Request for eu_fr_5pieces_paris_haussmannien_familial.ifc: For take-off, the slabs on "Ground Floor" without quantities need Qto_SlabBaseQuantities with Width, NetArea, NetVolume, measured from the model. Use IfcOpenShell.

First a look at what the model holds.

```python
import ifcopenshell
import ifcopenshell.util.element
import ifcopenshell.util.unit

model = ifcopenshell.open("eu_fr_5pieces_paris_haussmannien_familial.ifc")
print(model.schema)
for unit_type in ("LENGTHUNIT", "AREAUNIT", "VOLUMEUNIT"):
    print(unit_type, ifcopenshell.util.unit.calculate_unit_scale(model, unit_type))
storey = next(s for s in model.by_type("IfcBuildingStorey") if s.Name == "Ground Floor")
slabs = [e for e in ifcopenshell.util.element.get_decomposition(storey) if e.is_a("IfcSlab")]
for e in sorted(slabs, key=lambda e: e.id()):
    print(e.id(), e.is_a(), e.Name, list(ifcopenshell.util.element.get_psets(e, qtos_only=True)), sep=" | ")
```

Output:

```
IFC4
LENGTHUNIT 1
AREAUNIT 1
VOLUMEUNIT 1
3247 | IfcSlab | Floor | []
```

```python
import ifcopenshell
import ifcopenshell.api.pset
import ifcopenshell.geom
import ifcopenshell.util.element
import ifcopenshell.util.shape
import ifcopenshell.util.unit

model = ifcopenshell.open("eu_fr_5pieces_paris_haussmannien_familial.ifc")
unit_scale = ifcopenshell.util.unit.calculate_unit_scale(model)
area_scale = ifcopenshell.util.unit.calculate_unit_scale(model, "AREAUNIT")
volume_scale = ifcopenshell.util.unit.calculate_unit_scale(model, "VOLUMEUNIT")
settings = ifcopenshell.geom.settings()

storey = next(s for s in model.by_type("IfcBuildingStorey") if s.Name == "Ground Floor")
slabs = [e for e in ifcopenshell.util.element.get_decomposition(storey) if e.is_a("IfcSlab")]

for e in sorted(slabs, key=lambda e: e.id()):
    if ifcopenshell.util.element.get_psets(e, qtos_only=True, should_inherit=False):
        continue
    # Geometry comes back in metres, in the element's own axes.
    shape = ifcopenshell.geom.create_shape(settings, e)
    values = {
        "Width": ifcopenshell.util.shape.get_z(shape.geometry) / unit_scale,
        "NetArea": ifcopenshell.util.shape.get_footprint_area(shape.geometry) / area_scale,
        "NetVolume": ifcopenshell.util.shape.get_volume(shape.geometry) / volume_scale,
    }
    qto = ifcopenshell.api.pset.add_qto(model, product=e, name="Qto_SlabBaseQuantities")
    ifcopenshell.api.pset.edit_qto(model, qto=qto, properties=values)
    print(e.id(), {k: round(v, 3) for k, v in values.items()})

model.write("eu_fr_5pieces_paris_haussmannien_familial_v2.ifc")
```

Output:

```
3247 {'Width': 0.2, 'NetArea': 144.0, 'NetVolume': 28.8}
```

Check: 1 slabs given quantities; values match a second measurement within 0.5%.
